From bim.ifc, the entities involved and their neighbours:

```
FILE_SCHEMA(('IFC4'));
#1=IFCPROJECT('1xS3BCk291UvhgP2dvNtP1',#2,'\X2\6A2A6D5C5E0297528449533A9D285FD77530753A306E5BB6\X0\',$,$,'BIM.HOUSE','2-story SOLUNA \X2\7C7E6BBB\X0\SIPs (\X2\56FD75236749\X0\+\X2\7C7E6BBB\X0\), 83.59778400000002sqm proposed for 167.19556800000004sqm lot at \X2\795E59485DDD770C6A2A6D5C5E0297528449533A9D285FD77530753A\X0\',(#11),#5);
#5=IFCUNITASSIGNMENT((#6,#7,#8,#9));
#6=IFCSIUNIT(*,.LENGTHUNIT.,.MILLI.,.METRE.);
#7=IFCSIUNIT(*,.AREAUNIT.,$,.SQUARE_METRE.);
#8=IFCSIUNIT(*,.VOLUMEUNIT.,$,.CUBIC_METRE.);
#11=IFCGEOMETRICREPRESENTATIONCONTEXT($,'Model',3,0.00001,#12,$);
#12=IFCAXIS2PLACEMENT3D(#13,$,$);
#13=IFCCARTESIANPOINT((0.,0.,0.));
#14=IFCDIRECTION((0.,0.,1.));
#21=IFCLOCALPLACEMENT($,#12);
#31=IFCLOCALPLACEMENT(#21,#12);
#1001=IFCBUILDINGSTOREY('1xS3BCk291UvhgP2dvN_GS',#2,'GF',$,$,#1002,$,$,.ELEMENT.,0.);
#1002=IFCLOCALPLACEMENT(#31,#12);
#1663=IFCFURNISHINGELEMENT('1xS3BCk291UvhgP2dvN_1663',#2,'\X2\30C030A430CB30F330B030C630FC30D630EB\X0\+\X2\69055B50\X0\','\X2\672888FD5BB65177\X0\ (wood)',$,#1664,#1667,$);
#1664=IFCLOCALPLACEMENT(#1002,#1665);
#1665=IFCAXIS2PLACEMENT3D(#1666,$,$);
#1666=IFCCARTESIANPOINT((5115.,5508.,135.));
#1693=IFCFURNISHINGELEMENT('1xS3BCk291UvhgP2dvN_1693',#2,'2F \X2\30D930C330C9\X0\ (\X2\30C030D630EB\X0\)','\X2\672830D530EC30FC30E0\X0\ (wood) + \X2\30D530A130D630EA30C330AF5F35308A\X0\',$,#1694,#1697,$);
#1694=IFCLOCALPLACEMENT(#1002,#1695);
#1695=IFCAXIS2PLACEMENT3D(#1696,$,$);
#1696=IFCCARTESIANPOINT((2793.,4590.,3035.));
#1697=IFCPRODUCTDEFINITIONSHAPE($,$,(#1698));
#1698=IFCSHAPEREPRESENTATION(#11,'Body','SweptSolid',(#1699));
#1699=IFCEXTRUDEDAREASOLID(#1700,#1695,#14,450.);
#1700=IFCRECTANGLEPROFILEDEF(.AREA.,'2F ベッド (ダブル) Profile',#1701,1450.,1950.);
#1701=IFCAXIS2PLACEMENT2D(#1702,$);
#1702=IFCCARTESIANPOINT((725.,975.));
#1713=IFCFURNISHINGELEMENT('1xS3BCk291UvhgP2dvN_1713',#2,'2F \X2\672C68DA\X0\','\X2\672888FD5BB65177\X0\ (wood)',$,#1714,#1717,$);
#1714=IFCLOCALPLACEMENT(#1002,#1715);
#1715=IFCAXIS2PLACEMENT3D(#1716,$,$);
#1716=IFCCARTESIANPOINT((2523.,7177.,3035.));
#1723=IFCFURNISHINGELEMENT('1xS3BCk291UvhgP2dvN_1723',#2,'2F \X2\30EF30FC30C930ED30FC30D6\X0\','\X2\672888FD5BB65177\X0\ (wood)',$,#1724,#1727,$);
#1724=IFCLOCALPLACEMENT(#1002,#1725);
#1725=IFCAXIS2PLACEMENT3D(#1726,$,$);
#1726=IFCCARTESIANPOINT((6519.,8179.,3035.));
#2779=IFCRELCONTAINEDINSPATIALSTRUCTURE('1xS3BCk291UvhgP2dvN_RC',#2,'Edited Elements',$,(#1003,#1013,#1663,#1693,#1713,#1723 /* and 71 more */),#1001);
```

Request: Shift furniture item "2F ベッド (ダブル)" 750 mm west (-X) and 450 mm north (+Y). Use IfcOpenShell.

```python
import ifcopenshell
import ifcopenshell.api.geometry
import ifcopenshell.util.placement

model = ifcopenshell.open("bim.ifc")

item = model.by_guid("1xS3BCk291UvhgP2dvN_1693")
matrix = ifcopenshell.util.placement.get_local_placement(item.ObjectPlacement)
matrix[0, 3] -= 750.0
matrix[1, 3] += 450.0
ifcopenshell.api.geometry.edit_object_placement(model, product=item, matrix=matrix, is_si=False)

print(ifcopenshell.util.placement.get_local_placement(item.ObjectPlacement).round(3) + 0.0)

model.write("bim_updated.ifc")
```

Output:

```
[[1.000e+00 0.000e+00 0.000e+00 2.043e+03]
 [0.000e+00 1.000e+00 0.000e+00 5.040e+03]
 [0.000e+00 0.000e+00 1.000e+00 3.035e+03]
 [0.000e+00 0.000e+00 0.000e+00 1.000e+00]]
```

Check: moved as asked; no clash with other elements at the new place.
